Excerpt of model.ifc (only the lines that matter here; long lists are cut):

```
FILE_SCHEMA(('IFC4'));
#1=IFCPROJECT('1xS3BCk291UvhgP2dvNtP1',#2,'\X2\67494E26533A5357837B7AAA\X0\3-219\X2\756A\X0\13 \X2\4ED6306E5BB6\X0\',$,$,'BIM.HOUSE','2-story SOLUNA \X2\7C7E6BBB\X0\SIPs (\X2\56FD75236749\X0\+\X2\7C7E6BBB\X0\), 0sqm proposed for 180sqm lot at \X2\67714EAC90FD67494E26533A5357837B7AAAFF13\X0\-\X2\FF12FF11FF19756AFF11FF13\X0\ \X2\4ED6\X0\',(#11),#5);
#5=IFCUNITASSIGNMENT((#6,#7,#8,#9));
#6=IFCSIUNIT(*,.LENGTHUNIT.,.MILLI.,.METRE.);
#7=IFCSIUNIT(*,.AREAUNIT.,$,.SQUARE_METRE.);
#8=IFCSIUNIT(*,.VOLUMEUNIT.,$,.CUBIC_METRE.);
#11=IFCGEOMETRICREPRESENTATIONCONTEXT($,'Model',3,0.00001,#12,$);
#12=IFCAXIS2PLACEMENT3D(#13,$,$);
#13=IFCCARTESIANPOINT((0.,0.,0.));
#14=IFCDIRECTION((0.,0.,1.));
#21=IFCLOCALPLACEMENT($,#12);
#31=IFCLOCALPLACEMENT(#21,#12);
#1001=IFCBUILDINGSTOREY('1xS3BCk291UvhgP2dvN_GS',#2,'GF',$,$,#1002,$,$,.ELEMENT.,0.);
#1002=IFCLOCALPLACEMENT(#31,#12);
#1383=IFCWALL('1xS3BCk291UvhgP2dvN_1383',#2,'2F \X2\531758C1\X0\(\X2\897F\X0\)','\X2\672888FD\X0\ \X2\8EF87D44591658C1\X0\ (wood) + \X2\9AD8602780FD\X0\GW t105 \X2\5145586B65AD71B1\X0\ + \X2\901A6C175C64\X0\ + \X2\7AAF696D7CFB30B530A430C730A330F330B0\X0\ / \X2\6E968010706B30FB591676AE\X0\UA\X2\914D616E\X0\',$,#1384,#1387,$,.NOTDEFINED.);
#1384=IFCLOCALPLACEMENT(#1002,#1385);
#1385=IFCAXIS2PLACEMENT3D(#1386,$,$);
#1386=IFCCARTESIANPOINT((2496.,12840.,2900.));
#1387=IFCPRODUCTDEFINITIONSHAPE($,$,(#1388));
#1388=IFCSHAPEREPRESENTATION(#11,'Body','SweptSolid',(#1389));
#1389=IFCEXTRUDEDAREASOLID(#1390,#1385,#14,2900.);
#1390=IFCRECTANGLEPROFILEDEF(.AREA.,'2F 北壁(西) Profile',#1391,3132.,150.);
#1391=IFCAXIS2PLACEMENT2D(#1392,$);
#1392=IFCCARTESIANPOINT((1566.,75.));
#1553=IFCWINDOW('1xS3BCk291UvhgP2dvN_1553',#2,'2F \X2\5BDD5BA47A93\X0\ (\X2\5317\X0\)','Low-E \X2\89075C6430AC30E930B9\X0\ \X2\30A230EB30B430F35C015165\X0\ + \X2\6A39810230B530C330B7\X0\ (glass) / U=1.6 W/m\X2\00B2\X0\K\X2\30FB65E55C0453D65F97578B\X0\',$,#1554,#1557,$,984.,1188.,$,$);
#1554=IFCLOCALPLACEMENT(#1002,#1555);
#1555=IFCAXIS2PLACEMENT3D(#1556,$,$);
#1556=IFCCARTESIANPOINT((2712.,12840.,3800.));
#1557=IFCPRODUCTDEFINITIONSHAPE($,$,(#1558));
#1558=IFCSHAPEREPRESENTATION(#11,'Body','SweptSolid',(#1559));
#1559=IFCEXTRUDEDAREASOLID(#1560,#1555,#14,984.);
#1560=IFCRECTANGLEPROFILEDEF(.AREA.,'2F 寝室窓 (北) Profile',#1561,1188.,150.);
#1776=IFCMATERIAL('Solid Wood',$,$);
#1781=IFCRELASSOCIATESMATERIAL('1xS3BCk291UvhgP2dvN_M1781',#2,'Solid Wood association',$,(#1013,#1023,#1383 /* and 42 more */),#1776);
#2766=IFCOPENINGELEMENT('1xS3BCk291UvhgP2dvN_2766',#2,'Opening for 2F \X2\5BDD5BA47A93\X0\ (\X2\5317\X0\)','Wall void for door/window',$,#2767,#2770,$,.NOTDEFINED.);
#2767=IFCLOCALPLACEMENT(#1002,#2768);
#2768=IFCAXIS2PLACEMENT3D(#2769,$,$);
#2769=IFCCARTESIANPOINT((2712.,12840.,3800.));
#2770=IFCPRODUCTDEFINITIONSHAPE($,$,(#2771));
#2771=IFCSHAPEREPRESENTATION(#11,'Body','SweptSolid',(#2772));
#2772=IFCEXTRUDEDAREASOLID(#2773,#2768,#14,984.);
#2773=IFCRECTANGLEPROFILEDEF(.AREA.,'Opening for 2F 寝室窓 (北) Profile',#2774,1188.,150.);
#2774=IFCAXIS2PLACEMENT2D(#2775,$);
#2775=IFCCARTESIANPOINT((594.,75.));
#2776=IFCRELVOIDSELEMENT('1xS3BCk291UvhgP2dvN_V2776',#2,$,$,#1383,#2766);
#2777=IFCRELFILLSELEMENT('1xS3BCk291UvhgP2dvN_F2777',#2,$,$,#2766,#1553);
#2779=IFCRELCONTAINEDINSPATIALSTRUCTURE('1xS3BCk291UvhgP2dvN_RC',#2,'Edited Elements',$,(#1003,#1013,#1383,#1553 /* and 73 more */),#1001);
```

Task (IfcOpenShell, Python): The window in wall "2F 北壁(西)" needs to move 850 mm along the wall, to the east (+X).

```python
import ifcopenshell
import ifcopenshell.api.geometry
import ifcopenshell.util.placement
import ifcopenshell.util.unit

model = ifcopenshell.open("model.ifc")
unit_scale = ifcopenshell.util.unit.calculate_unit_scale(model)

window = model.by_guid("1xS3BCk291UvhgP2dvN_1553")
opening = window.FillsVoids[0].RelatingOpeningElement
wall = opening.VoidsElements[0].RelatingBuildingElement

wall_matrix = ifcopenshell.util.placement.get_local_placement(wall.ObjectPlacement)
shift = wall_matrix[:3, 0] * 0.85 / unit_scale
before = ifcopenshell.util.placement.get_local_placement(window.ObjectPlacement)[:3, 3].copy()

# The window is not placed relative to its opening, so move both.
for product in (opening, window):
    matrix = ifcopenshell.util.placement.get_local_placement(product.ObjectPlacement)
    matrix[:3, 3] += shift
    ifcopenshell.api.geometry.edit_object_placement(model, product=product, matrix=matrix, is_si=False)

after = ifcopenshell.util.placement.get_local_placement(window.ObjectPlacement)[:3, 3]
print("window moved by", (after - before).round(3) + 0.0)

model.write("model_updated.ifc")
```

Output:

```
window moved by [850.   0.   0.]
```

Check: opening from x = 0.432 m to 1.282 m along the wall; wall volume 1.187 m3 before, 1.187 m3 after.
